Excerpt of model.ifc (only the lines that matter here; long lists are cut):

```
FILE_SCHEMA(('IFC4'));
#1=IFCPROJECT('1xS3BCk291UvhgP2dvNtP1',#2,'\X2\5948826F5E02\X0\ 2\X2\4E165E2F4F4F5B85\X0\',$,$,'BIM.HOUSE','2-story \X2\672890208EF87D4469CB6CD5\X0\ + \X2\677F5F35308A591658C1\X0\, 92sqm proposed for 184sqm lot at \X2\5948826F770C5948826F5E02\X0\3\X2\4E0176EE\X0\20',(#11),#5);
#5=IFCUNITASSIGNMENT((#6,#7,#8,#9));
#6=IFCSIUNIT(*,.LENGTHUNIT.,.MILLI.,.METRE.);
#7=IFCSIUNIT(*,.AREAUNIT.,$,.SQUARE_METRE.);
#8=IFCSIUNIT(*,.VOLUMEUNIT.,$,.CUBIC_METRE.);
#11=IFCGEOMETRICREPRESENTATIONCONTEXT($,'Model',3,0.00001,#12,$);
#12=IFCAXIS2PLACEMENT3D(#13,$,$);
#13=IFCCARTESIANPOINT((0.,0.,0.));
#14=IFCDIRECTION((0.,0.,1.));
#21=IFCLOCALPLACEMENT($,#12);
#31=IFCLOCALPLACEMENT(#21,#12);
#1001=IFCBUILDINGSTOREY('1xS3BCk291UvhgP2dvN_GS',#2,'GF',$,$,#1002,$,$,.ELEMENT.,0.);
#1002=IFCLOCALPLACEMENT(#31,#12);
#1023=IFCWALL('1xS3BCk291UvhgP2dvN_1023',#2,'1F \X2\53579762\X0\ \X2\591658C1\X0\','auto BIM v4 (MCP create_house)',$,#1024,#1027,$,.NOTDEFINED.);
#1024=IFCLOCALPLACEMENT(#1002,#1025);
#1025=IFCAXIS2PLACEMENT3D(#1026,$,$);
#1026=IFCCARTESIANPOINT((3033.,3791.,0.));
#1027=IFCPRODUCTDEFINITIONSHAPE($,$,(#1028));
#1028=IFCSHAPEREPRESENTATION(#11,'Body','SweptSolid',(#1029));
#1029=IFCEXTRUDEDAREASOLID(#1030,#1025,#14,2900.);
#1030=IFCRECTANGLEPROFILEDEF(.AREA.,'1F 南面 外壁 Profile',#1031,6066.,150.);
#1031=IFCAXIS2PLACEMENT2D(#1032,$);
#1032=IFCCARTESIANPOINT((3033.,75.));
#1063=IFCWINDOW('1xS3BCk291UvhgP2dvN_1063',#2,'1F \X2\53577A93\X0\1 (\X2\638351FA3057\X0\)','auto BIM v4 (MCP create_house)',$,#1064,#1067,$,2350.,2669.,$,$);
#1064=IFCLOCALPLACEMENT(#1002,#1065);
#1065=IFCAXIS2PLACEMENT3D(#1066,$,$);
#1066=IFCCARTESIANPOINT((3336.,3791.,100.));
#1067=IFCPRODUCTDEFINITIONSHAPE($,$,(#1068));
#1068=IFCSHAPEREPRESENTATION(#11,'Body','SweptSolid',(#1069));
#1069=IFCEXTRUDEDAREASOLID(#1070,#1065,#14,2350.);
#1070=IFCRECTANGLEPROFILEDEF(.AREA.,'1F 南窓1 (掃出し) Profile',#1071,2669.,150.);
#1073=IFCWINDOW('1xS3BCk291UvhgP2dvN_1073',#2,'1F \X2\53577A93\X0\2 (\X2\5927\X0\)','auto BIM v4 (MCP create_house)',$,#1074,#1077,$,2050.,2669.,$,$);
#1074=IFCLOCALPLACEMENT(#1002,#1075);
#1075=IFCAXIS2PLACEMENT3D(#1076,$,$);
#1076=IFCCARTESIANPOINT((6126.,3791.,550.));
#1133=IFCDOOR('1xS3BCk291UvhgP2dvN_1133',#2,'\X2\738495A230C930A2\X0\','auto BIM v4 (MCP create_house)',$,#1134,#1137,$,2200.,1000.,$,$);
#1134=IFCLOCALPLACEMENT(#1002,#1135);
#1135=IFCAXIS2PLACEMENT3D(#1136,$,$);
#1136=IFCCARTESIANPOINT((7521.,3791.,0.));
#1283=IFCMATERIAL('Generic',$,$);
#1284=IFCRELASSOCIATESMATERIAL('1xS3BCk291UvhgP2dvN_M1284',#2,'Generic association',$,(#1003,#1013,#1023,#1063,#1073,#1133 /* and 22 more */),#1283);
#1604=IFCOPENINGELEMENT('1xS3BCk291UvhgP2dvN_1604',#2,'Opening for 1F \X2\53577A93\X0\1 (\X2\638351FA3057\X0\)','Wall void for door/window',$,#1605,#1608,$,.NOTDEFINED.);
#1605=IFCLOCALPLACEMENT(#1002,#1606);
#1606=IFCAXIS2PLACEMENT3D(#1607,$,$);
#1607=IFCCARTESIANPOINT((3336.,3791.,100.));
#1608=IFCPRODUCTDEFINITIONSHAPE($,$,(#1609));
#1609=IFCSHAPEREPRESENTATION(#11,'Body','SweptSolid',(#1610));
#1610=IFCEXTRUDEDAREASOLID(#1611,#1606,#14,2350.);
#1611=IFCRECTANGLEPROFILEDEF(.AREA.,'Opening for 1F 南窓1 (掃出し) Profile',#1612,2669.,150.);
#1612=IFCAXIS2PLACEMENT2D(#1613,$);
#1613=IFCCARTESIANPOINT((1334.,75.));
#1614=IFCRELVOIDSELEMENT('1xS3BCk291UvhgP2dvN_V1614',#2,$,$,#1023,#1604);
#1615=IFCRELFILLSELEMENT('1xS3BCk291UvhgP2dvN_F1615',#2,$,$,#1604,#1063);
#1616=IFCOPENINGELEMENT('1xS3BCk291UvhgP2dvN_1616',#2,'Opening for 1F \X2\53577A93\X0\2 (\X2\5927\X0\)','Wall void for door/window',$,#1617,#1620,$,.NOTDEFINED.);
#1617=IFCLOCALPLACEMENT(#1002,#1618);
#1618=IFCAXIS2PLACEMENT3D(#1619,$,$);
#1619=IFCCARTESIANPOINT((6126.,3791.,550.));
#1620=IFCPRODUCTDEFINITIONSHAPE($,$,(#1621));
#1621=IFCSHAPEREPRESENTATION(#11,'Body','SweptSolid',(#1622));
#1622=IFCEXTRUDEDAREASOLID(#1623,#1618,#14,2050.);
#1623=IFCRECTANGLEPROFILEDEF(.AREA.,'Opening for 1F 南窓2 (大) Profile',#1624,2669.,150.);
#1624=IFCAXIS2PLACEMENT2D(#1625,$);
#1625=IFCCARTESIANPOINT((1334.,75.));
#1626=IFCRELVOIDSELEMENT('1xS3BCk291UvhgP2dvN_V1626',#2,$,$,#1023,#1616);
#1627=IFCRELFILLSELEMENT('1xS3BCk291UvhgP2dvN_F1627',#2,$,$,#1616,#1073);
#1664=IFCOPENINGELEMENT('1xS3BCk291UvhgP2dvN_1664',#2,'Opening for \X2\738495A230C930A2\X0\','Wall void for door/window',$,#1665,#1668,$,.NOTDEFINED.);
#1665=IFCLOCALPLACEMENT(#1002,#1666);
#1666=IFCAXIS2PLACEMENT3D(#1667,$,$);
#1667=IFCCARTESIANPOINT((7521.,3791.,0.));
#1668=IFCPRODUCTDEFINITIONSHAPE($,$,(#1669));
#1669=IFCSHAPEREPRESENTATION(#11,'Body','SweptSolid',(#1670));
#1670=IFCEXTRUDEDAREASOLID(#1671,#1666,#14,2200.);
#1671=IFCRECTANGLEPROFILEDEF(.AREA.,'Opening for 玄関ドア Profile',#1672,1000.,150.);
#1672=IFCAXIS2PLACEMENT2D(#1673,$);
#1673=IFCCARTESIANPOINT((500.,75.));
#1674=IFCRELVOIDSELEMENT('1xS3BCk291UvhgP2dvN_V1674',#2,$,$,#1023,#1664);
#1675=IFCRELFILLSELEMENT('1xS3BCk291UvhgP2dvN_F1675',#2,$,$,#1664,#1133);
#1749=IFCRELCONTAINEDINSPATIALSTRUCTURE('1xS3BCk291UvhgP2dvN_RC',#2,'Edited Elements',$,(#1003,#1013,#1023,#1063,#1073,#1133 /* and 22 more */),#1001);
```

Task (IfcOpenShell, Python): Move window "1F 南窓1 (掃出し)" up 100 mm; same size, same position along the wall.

```python
import numpy as np
import ifcopenshell
import ifcopenshell.api.geometry
import ifcopenshell.util.placement
import ifcopenshell.util.unit

model = ifcopenshell.open("model.ifc")
unit_scale = ifcopenshell.util.unit.calculate_unit_scale(model)

window = model.by_id(1063)
opening = window.FillsVoids[0].RelatingOpeningElement
dz = 0.1 / unit_scale

shift = np.array([0.0, 0.0, dz])
# The window is not placed relative to its opening, so move both.
for product in (opening, window):
    matrix = ifcopenshell.util.placement.get_local_placement(product.ObjectPlacement)
    matrix[:3, 3] += shift
    ifcopenshell.api.geometry.edit_object_placement(model, product=product, matrix=matrix, is_si=False)

print(f"moved by {dz * unit_scale:+.3f} m")

model.write("model_edited.ifc")
```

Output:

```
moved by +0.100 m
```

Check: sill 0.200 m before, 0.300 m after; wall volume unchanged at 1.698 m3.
